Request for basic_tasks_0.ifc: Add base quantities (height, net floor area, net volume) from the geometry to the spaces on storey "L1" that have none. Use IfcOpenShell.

First a look at what the model holds.

```python
import ifcopenshell
import ifcopenshell.util.element
import ifcopenshell.util.unit

model = ifcopenshell.open("basic_tasks_0.ifc")
print(model.schema)
for unit_type in ("LENGTHUNIT", "AREAUNIT", "VOLUMEUNIT"):
    print(unit_type, ifcopenshell.util.unit.calculate_unit_scale(model, unit_type))
storey = next(s for s in model.by_type("IfcBuildingStorey") if s.Name == "L1")
spaces = [e for e in ifcopenshell.util.element.get_decomposition(storey) if e.is_a("IfcSpace")]
for e in sorted(spaces, key=lambda e: e.id()):
    print(e.id(), e.is_a(), e.Name, list(ifcopenshell.util.element.get_psets(e, qtos_only=True)), sep=" | ")
```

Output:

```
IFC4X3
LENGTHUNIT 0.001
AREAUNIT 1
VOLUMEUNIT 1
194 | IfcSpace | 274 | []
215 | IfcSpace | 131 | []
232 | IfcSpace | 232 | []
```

```python
import ifcopenshell
import ifcopenshell.api.pset
import ifcopenshell.geom
import ifcopenshell.util.element
import ifcopenshell.util.shape
import ifcopenshell.util.unit

model = ifcopenshell.open("basic_tasks_0.ifc")
unit_scale = ifcopenshell.util.unit.calculate_unit_scale(model)
area_scale = ifcopenshell.util.unit.calculate_unit_scale(model, "AREAUNIT")
volume_scale = ifcopenshell.util.unit.calculate_unit_scale(model, "VOLUMEUNIT")
settings = ifcopenshell.geom.settings()

storey = next(s for s in model.by_type("IfcBuildingStorey") if s.Name == "L1")
spaces = [e for e in ifcopenshell.util.element.get_decomposition(storey) if e.is_a("IfcSpace")]

for e in sorted(spaces, key=lambda e: e.id()):
    if ifcopenshell.util.element.get_psets(e, qtos_only=True, should_inherit=False):
        continue
    # Geometry comes back in metres, in the element's own axes.
    shape = ifcopenshell.geom.create_shape(settings, e)
    values = {
        "Height": ifcopenshell.util.shape.get_z(shape.geometry) / unit_scale,
        "NetFloorArea": ifcopenshell.util.shape.get_footprint_area(shape.geometry) / area_scale,
        "NetVolume": ifcopenshell.util.shape.get_volume(shape.geometry) / volume_scale,
    }
    qto = ifcopenshell.api.pset.add_qto(model, product=e, name="Qto_SpaceBaseQuantities")
    ifcopenshell.api.pset.edit_qto(model, qto=qto, properties=values)
    print(e.id(), {k: round(v, 3) for k, v in values.items()})

model.write("basic_tasks_0_rev.ifc")
```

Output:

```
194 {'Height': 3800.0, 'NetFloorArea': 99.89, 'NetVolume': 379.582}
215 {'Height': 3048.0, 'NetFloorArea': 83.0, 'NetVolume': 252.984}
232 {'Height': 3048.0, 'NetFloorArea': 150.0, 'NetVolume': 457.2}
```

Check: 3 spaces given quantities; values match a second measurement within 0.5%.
